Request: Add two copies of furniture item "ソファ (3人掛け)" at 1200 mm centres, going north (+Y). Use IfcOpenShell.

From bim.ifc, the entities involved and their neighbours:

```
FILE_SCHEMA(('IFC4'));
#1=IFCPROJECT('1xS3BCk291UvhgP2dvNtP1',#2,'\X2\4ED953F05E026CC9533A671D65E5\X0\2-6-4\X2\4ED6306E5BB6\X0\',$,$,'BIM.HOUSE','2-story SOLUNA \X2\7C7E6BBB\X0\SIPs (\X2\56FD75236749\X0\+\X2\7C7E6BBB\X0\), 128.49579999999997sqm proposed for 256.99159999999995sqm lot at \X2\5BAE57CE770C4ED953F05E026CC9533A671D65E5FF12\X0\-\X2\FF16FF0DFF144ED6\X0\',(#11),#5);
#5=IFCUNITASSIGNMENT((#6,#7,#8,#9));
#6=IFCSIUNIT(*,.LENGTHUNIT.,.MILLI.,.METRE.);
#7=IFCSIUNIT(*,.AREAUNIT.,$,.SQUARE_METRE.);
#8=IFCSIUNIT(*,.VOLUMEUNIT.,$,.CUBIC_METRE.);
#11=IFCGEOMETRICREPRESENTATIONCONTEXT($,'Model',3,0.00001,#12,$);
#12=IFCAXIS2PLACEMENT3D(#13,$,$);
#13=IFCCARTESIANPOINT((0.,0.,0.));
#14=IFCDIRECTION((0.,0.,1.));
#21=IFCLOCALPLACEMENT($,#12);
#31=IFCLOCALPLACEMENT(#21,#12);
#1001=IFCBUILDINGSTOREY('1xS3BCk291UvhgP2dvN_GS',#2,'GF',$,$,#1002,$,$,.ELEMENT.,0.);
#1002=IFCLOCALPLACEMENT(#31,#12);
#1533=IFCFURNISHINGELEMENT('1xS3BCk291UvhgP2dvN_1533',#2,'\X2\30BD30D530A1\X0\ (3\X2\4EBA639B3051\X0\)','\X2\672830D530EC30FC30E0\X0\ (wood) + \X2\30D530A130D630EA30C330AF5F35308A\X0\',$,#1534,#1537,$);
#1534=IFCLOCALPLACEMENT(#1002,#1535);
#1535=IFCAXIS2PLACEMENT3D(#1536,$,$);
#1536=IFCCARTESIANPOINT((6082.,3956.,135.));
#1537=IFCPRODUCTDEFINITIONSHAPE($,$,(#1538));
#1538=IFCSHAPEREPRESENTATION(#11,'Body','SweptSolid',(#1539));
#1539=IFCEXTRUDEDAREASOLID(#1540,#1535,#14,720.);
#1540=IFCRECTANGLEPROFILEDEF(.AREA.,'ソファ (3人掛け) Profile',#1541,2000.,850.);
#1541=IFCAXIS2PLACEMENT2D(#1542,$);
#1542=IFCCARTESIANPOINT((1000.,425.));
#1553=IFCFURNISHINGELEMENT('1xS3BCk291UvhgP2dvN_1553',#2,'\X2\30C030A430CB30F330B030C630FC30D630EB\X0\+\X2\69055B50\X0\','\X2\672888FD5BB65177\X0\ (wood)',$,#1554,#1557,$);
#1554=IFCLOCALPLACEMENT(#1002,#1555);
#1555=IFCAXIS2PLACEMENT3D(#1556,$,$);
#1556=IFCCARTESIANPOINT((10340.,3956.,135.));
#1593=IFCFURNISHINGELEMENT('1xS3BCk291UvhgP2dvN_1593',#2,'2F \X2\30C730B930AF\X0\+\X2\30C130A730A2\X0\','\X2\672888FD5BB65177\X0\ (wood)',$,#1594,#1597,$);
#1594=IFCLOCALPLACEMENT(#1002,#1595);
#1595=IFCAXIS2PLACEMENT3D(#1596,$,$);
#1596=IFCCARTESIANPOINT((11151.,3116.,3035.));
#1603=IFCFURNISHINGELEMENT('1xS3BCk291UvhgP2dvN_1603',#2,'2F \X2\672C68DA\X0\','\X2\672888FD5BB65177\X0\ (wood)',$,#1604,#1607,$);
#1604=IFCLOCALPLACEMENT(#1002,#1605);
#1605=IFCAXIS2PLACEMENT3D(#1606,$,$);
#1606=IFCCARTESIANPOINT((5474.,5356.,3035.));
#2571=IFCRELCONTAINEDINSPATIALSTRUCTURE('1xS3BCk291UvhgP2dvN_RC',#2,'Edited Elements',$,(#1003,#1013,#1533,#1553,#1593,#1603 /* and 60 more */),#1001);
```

```python
import numpy as np
import ifcopenshell
import ifcopenshell.api.geometry
import ifcopenshell.api.root
import ifcopenshell.util.element
import ifcopenshell.util.placement

model = ifcopenshell.open("bim.ifc")


def reuse_history(source, copy):
    """copy_class also copies each property set's owner history, people and application; keep the originals."""
    for rel in copy.IsDefinedBy:
        if rel.is_a("IfcRelDefinesByProperties") and (history := rel.RelatingPropertyDefinition.OwnerHistory):
            rel.RelatingPropertyDefinition.OwnerHistory = source.OwnerHistory
            ifcopenshell.util.element.remove_deep2(model, history)


source = model.by_guid("1xS3BCk291UvhgP2dvN_1533")
base = ifcopenshell.util.placement.get_local_placement(source.ObjectPlacement)
step = np.array([0.0, 1.0, 0.0]) * 1200.0

for i in range(1, 3):
    copy = ifcopenshell.api.root.copy_class(model, product=source)
    copy.Representation = ifcopenshell.util.element.copy_deep(
        model, source.Representation, exclude=["IfcGeometricRepresentationContext", "IfcRepresentationMap"]
    )
    reuse_history(source, copy)
    matrix = base.copy()
    matrix[:3, 3] += i * step
    print("added at", matrix[:3, 3].round(3) + 0.0)
    ifcopenshell.api.geometry.edit_object_placement(model, product=copy, matrix=matrix, is_si=False)

model.write("bim_rev.ifc")
```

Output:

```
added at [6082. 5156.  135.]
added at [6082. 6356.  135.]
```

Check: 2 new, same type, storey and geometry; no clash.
